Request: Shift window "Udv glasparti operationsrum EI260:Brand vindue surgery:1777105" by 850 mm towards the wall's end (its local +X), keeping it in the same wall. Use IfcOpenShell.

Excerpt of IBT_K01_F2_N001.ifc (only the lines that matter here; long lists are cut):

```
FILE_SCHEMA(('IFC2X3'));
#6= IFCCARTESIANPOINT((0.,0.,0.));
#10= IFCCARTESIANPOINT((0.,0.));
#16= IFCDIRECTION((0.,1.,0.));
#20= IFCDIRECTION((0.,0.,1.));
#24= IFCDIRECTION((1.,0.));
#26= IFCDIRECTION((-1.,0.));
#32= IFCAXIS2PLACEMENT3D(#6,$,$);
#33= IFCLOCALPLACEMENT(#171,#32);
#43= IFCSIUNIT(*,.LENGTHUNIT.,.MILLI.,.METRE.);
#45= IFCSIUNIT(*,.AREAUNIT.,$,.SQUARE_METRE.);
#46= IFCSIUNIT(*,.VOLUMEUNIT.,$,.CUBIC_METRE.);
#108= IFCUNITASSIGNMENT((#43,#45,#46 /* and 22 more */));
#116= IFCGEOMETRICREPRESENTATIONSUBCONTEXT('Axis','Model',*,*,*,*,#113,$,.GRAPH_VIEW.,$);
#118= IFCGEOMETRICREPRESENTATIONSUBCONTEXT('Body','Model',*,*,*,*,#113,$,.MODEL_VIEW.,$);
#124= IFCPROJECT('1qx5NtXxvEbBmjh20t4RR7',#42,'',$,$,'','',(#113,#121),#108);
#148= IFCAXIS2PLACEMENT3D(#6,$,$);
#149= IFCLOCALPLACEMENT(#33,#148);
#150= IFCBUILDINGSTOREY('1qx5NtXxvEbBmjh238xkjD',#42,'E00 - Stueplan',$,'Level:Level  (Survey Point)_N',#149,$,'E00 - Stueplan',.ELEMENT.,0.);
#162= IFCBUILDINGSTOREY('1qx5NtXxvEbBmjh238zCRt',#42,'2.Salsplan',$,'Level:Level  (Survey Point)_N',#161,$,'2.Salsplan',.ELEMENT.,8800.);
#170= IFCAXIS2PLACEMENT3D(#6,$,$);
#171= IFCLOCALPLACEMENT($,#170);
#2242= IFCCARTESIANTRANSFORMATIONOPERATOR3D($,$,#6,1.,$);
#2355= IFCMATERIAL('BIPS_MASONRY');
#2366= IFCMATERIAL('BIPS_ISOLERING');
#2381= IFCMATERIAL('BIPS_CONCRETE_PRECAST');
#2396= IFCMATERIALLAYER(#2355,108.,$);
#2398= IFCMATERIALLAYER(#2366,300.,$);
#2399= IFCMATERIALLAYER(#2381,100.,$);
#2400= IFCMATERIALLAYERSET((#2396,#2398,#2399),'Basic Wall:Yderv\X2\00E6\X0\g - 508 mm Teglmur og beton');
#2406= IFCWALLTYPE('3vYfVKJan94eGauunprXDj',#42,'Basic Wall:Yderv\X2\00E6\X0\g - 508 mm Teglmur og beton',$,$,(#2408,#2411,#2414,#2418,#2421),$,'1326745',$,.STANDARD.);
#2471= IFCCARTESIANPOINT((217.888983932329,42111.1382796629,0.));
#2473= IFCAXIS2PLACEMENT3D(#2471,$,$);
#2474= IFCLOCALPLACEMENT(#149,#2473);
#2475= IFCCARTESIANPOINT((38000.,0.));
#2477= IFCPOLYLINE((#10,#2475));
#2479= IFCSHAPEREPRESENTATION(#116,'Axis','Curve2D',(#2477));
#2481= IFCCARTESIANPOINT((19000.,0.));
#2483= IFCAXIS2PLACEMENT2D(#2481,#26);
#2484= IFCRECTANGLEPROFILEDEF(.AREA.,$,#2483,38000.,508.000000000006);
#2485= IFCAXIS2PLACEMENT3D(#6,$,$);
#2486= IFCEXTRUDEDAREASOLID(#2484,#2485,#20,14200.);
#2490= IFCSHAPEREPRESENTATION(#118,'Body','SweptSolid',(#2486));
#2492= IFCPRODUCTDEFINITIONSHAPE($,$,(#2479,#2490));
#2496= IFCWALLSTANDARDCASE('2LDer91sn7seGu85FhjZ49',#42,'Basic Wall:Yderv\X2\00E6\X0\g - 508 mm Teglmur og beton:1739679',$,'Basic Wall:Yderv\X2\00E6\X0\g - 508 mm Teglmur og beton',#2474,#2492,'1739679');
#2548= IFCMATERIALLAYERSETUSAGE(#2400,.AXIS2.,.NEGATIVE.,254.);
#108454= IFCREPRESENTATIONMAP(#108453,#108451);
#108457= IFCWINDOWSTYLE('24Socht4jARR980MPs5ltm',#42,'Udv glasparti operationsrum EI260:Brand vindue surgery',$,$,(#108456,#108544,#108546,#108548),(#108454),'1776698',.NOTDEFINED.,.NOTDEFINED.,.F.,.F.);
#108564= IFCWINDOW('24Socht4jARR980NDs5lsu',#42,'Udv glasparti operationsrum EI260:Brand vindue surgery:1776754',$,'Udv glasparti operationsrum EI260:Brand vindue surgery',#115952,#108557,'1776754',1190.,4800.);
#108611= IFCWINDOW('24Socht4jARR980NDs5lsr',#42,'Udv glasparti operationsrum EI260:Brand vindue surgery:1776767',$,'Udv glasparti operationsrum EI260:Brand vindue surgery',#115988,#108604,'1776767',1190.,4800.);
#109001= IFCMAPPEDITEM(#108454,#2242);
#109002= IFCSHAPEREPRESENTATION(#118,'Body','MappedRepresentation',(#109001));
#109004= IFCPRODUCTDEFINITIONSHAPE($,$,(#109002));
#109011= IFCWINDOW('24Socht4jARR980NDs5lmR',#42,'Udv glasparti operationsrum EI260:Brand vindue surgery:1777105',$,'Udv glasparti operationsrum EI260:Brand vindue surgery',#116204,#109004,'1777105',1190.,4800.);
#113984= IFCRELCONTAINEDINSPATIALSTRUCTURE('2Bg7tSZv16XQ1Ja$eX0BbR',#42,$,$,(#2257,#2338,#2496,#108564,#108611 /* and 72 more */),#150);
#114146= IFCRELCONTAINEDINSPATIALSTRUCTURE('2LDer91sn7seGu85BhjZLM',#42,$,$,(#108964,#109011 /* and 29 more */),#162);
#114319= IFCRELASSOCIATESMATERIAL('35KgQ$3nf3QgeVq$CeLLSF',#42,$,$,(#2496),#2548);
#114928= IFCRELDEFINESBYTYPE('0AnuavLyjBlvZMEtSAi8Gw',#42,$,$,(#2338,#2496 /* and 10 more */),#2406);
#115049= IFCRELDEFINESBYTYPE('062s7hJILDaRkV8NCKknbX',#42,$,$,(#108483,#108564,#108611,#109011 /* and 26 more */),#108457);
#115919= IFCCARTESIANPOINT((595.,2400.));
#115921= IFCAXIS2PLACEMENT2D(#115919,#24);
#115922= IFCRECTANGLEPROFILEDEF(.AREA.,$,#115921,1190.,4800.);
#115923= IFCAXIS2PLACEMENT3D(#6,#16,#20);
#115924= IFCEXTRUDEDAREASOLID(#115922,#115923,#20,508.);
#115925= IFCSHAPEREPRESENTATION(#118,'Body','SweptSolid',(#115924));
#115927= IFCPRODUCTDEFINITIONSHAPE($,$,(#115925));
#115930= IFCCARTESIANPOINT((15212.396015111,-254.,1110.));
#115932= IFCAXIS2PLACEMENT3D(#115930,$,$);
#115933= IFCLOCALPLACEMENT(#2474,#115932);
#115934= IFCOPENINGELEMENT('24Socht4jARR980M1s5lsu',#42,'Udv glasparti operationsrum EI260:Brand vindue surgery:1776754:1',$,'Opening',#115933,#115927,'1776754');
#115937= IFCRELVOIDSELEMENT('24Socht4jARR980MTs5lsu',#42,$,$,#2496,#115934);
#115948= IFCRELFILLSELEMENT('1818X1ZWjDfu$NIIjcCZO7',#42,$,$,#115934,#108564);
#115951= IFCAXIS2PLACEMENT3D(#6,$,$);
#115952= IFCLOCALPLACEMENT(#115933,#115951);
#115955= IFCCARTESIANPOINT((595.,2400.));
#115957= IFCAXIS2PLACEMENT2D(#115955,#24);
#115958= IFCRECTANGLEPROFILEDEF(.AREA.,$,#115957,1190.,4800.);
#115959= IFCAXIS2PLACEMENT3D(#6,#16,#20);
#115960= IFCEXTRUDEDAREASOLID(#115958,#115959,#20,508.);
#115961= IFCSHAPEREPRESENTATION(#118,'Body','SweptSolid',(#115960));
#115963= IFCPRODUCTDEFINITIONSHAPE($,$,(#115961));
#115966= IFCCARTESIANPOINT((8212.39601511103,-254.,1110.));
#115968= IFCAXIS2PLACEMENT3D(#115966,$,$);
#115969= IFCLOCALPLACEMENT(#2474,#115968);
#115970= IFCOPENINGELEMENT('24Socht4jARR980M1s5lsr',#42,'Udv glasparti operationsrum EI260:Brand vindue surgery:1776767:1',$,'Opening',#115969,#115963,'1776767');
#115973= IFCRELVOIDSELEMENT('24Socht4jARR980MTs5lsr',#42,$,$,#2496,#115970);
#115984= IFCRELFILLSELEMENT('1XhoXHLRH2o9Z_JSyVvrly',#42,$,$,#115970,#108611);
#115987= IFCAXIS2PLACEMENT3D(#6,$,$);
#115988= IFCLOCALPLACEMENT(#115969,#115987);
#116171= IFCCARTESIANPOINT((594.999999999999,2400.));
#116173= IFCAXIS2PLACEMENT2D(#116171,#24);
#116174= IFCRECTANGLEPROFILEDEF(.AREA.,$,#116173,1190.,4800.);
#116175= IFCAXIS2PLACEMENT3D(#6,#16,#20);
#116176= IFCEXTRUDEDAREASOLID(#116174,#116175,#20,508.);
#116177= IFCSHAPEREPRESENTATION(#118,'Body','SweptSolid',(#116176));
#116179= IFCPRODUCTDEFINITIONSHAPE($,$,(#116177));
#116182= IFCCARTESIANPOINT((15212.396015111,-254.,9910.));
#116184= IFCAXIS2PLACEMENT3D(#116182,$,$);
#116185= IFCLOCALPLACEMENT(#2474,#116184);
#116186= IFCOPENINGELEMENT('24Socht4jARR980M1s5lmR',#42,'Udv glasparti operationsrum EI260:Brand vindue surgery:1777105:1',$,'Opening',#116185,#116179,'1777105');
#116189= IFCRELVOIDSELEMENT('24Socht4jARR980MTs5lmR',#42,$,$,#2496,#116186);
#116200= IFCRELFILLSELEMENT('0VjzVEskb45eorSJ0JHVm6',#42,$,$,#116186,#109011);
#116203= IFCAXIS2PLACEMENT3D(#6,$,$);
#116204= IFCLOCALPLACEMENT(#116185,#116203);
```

```python
import ifcopenshell
import ifcopenshell.api.geometry
import ifcopenshell.util.placement

model = ifcopenshell.open("IBT_K01_F2_N001.ifc")

window = model.by_guid("24Socht4jARR980NDs5lmR")
opening = window.FillsVoids[0].RelatingOpeningElement
wall = opening.VoidsElements[0].RelatingBuildingElement

wall_matrix = ifcopenshell.util.placement.get_local_placement(wall.ObjectPlacement)
shift = wall_matrix[:3, 0] * 850.0
before = ifcopenshell.util.placement.get_local_placement(window.ObjectPlacement)[:3, 3].copy()

# The window is placed relative to its opening, so it follows when the opening moves.
matrix = ifcopenshell.util.placement.get_local_placement(opening.ObjectPlacement)
matrix[:3, 3] += shift
ifcopenshell.api.geometry.edit_object_placement(
    model, product=opening, matrix=matrix, is_si=False, should_transform_children=True
)

after = ifcopenshell.util.placement.get_local_placement(window.ObjectPlacement)[:3, 3]
print("window moved by", (after - before).round(3) + 0.0)

model.write("IBT_K01_F2_N001-out.ifc")
```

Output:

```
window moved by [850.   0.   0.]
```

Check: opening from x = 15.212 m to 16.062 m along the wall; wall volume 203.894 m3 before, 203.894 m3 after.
